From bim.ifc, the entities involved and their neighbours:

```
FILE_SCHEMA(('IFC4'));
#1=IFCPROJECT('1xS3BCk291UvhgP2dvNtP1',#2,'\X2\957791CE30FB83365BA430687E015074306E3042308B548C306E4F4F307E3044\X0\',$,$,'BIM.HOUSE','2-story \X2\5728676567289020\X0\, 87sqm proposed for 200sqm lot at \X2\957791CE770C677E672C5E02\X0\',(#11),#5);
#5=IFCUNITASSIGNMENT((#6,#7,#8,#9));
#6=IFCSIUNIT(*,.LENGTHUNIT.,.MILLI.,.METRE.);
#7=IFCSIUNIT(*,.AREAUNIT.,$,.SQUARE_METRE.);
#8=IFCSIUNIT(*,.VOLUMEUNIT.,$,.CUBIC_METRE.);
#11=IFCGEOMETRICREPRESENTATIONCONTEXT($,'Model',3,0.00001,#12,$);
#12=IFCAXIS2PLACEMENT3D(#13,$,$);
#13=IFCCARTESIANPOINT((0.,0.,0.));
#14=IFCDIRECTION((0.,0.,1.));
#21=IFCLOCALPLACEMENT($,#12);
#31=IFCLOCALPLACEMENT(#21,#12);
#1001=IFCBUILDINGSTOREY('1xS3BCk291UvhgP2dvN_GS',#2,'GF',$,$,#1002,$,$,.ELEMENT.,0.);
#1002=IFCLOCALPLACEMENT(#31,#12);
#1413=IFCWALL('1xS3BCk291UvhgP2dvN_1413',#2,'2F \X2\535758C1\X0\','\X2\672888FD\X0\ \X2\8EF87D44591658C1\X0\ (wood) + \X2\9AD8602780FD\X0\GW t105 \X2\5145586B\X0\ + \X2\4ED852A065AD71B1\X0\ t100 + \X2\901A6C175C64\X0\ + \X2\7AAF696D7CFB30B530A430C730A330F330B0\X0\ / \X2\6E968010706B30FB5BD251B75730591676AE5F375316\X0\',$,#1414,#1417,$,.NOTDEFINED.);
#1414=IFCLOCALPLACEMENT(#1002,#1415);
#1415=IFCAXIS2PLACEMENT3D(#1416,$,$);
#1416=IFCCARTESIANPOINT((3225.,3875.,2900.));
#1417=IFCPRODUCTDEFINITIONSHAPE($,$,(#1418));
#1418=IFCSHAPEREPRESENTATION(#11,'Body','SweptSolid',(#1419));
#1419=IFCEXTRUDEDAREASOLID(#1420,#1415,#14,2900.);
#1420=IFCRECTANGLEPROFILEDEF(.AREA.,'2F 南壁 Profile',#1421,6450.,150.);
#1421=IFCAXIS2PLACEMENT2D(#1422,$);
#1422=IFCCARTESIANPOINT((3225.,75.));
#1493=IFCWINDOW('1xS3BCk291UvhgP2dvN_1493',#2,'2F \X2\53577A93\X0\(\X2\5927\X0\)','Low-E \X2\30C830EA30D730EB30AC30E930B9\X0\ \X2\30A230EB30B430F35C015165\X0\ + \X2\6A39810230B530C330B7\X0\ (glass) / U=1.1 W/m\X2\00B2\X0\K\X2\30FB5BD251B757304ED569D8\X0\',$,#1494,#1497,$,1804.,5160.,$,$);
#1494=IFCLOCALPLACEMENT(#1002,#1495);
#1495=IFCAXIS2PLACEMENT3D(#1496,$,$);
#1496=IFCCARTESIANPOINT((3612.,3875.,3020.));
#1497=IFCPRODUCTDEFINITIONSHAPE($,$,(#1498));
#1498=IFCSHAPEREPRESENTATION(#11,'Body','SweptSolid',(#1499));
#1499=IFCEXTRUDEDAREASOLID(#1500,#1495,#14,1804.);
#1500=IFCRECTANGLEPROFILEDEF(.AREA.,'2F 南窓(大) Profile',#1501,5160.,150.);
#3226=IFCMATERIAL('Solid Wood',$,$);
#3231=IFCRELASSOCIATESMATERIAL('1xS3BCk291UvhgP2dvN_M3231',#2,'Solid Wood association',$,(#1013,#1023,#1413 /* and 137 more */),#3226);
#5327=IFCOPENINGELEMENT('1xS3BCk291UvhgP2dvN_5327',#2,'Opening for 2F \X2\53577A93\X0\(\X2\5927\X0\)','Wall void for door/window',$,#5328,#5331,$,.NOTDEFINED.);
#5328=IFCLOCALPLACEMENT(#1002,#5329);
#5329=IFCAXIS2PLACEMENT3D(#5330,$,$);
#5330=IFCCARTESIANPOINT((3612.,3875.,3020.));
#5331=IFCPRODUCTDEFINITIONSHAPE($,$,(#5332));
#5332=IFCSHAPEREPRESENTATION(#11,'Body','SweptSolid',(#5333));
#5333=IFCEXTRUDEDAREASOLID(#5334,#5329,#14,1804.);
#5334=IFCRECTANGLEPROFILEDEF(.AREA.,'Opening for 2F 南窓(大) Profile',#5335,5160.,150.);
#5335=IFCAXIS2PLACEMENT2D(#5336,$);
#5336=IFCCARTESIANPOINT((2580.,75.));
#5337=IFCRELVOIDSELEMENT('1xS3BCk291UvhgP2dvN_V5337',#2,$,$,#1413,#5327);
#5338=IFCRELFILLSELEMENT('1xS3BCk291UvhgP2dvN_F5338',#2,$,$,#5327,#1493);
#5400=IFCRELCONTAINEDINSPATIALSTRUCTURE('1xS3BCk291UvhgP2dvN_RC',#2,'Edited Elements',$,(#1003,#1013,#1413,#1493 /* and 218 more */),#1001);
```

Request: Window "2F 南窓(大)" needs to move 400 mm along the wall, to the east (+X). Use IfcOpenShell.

```python
import ifcopenshell
import ifcopenshell.api.geometry
import ifcopenshell.util.placement
import ifcopenshell.util.unit

model = ifcopenshell.open("bim.ifc")
unit_scale = ifcopenshell.util.unit.calculate_unit_scale(model)

window = model.by_id(1493)
opening = window.FillsVoids[0].RelatingOpeningElement
wall = opening.VoidsElements[0].RelatingBuildingElement

wall_matrix = ifcopenshell.util.placement.get_local_placement(wall.ObjectPlacement)
shift = wall_matrix[:3, 0] * 0.4 / unit_scale
before = ifcopenshell.util.placement.get_local_placement(window.ObjectPlacement)[:3, 3].copy()

# The window is not placed relative to its opening, so move both.
for product in (opening, window):
    matrix = ifcopenshell.util.placement.get_local_placement(product.ObjectPlacement)
    matrix[:3, 3] += shift
    ifcopenshell.api.geometry.edit_object_placement(model, product=product, matrix=matrix, is_si=False)

after = ifcopenshell.util.placement.get_local_placement(window.ObjectPlacement)[:3, 3]
print("window moved by", (after - before).round(3) + 0.0)

model.write("bim_rev.ifc")
```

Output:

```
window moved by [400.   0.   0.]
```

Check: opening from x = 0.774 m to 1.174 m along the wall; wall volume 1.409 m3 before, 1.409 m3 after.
